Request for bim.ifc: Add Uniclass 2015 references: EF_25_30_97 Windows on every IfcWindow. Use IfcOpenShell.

First a look at what the model holds.

```python
import ifcopenshell

model = ifcopenshell.open("bim.ifc")
print(model.schema)
print("classifications:", [c.Name for c in model.by_type("IfcClassification")])
for ifc_class in ("IfcDoor", "IfcRoof", "IfcStair", "IfcWall", "IfcWindow"):
    print(ifc_class, len(model.by_type(ifc_class)))
```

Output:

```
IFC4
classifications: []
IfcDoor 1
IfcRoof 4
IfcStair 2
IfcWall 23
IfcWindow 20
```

```python
import ifcopenshell
import ifcopenshell.api.classification

model = ifcopenshell.open("bim.ifc")

system = ifcopenshell.api.classification.add_classification(model, classification="Uniclass 2015")

codes = {
    "IfcWindow": ("EF_25_30_97", "Windows"),
}
for ifc_class, (code, name) in codes.items():
    products = model.by_type(ifc_class)
    ifcopenshell.api.classification.add_reference(
        model, products=products, classification=system, identification=code, name=name
    )
    print(code, len(products))

model.write("bim_updated.ifc")
```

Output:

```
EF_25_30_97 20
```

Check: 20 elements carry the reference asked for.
